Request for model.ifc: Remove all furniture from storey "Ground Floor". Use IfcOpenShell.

First a look at what the model holds.

```python
import ifcopenshell
import ifcopenshell.util.element

model = ifcopenshell.open("model.ifc")
print(model.schema)
storey = next(s for s in model.by_type("IfcBuildingStorey") if s.Name == "Ground Floor")
furniture = [e for e in ifcopenshell.util.element.get_decomposition(storey) if e.is_a("IfcFurnishingElement")]
seen = {}
for e in furniture:
    element_type = ifcopenshell.util.element.get_type(e)
    name = element_type.Name if element_type not in (None, e) else None
    seen[name] = seen.get(name, 0) + 1
for name, count in sorted(seen.items(), key=str):
    print(count, "x", name)
```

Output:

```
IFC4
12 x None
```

```python
import ifcopenshell
import ifcopenshell.api.root
import ifcopenshell.util.element

model = ifcopenshell.open("model.ifc")

storey = next(s for s in model.by_type("IfcBuildingStorey") if s.Name == "Ground Floor")
furniture = [e for e in ifcopenshell.util.element.get_decomposition(storey) if e.is_a("IfcFurnishingElement")]

for e in furniture:
    ifcopenshell.api.root.remove_product(model, product=e)
print(len(furniture), "removed")

model.write("model_edited.ifc")
```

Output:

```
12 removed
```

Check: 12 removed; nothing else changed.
